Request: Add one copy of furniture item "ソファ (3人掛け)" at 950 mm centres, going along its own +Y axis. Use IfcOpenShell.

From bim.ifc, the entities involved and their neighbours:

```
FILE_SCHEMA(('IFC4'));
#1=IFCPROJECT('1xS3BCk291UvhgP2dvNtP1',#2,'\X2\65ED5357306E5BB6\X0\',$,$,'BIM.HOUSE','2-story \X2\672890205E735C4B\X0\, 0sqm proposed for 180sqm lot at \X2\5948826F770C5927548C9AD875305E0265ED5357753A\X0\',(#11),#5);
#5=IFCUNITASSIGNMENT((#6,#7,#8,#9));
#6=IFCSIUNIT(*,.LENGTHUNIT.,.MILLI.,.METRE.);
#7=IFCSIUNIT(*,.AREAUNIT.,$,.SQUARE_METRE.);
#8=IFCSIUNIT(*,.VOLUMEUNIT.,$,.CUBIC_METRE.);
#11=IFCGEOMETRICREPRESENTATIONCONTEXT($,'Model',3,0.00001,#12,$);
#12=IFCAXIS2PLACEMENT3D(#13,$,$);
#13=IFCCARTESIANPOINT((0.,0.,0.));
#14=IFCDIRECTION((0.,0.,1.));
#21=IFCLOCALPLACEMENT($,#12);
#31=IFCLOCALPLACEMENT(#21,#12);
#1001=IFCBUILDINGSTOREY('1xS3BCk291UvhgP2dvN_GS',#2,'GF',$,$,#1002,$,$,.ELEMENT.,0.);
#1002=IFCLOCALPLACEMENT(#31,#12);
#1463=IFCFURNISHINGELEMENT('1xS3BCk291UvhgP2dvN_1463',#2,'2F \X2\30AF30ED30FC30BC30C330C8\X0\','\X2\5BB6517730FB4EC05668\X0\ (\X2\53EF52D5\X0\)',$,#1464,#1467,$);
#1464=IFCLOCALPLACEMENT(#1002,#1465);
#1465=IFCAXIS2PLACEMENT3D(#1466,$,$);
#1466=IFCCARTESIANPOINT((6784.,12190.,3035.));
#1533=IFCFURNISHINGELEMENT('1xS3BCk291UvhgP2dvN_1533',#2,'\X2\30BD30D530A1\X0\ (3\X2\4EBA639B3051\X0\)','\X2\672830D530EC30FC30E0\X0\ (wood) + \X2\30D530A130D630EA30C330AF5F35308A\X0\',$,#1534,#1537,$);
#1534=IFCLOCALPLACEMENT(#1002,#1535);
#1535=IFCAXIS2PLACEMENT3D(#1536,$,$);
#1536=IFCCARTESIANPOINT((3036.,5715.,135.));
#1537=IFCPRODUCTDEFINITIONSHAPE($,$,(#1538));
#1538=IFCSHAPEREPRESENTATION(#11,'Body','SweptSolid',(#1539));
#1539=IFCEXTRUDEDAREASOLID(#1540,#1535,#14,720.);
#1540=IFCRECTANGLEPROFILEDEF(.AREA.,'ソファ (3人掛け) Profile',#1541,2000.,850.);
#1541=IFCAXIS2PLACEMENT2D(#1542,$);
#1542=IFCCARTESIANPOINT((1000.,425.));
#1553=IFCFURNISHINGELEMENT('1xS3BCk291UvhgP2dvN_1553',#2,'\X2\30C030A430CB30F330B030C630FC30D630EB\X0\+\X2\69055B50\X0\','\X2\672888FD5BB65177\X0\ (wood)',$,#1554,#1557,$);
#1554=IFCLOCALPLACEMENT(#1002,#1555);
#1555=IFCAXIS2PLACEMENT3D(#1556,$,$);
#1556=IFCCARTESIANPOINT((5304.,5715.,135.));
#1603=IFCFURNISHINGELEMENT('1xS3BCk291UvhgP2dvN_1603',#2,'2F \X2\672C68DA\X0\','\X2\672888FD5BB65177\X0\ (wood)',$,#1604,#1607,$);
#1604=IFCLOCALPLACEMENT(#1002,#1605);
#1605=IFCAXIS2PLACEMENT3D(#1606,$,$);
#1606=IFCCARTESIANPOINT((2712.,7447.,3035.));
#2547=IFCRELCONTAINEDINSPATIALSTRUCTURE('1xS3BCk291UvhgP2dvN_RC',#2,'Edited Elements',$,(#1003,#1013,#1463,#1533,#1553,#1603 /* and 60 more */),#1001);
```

```python
import ifcopenshell
import ifcopenshell.api.geometry
import ifcopenshell.api.root
import ifcopenshell.util.element
import ifcopenshell.util.placement

model = ifcopenshell.open("bim.ifc")


def reuse_history(source, copy):
    """copy_class also copies each property set's owner history, people and application; keep the originals."""
    for rel in copy.IsDefinedBy:
        if rel.is_a("IfcRelDefinesByProperties") and (history := rel.RelatingPropertyDefinition.OwnerHistory):
            rel.RelatingPropertyDefinition.OwnerHistory = source.OwnerHistory
            ifcopenshell.util.element.remove_deep2(model, history)


source = model.by_guid("1xS3BCk291UvhgP2dvN_1533")
base = ifcopenshell.util.placement.get_local_placement(source.ObjectPlacement)
step = base[:3, 1] * 950.0

for i in range(1, 2):
    copy = ifcopenshell.api.root.copy_class(model, product=source)
    copy.Representation = ifcopenshell.util.element.copy_deep(
        model, source.Representation, exclude=["IfcGeometricRepresentationContext", "IfcRepresentationMap"]
    )
    reuse_history(source, copy)
    matrix = base.copy()
    matrix[:3, 3] += i * step
    print("added at", matrix[:3, 3].round(3) + 0.0)
    ifcopenshell.api.geometry.edit_object_placement(model, product=copy, matrix=matrix, is_si=False)

model.write("bim_updated.ifc")
```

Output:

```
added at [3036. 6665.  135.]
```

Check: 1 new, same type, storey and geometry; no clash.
